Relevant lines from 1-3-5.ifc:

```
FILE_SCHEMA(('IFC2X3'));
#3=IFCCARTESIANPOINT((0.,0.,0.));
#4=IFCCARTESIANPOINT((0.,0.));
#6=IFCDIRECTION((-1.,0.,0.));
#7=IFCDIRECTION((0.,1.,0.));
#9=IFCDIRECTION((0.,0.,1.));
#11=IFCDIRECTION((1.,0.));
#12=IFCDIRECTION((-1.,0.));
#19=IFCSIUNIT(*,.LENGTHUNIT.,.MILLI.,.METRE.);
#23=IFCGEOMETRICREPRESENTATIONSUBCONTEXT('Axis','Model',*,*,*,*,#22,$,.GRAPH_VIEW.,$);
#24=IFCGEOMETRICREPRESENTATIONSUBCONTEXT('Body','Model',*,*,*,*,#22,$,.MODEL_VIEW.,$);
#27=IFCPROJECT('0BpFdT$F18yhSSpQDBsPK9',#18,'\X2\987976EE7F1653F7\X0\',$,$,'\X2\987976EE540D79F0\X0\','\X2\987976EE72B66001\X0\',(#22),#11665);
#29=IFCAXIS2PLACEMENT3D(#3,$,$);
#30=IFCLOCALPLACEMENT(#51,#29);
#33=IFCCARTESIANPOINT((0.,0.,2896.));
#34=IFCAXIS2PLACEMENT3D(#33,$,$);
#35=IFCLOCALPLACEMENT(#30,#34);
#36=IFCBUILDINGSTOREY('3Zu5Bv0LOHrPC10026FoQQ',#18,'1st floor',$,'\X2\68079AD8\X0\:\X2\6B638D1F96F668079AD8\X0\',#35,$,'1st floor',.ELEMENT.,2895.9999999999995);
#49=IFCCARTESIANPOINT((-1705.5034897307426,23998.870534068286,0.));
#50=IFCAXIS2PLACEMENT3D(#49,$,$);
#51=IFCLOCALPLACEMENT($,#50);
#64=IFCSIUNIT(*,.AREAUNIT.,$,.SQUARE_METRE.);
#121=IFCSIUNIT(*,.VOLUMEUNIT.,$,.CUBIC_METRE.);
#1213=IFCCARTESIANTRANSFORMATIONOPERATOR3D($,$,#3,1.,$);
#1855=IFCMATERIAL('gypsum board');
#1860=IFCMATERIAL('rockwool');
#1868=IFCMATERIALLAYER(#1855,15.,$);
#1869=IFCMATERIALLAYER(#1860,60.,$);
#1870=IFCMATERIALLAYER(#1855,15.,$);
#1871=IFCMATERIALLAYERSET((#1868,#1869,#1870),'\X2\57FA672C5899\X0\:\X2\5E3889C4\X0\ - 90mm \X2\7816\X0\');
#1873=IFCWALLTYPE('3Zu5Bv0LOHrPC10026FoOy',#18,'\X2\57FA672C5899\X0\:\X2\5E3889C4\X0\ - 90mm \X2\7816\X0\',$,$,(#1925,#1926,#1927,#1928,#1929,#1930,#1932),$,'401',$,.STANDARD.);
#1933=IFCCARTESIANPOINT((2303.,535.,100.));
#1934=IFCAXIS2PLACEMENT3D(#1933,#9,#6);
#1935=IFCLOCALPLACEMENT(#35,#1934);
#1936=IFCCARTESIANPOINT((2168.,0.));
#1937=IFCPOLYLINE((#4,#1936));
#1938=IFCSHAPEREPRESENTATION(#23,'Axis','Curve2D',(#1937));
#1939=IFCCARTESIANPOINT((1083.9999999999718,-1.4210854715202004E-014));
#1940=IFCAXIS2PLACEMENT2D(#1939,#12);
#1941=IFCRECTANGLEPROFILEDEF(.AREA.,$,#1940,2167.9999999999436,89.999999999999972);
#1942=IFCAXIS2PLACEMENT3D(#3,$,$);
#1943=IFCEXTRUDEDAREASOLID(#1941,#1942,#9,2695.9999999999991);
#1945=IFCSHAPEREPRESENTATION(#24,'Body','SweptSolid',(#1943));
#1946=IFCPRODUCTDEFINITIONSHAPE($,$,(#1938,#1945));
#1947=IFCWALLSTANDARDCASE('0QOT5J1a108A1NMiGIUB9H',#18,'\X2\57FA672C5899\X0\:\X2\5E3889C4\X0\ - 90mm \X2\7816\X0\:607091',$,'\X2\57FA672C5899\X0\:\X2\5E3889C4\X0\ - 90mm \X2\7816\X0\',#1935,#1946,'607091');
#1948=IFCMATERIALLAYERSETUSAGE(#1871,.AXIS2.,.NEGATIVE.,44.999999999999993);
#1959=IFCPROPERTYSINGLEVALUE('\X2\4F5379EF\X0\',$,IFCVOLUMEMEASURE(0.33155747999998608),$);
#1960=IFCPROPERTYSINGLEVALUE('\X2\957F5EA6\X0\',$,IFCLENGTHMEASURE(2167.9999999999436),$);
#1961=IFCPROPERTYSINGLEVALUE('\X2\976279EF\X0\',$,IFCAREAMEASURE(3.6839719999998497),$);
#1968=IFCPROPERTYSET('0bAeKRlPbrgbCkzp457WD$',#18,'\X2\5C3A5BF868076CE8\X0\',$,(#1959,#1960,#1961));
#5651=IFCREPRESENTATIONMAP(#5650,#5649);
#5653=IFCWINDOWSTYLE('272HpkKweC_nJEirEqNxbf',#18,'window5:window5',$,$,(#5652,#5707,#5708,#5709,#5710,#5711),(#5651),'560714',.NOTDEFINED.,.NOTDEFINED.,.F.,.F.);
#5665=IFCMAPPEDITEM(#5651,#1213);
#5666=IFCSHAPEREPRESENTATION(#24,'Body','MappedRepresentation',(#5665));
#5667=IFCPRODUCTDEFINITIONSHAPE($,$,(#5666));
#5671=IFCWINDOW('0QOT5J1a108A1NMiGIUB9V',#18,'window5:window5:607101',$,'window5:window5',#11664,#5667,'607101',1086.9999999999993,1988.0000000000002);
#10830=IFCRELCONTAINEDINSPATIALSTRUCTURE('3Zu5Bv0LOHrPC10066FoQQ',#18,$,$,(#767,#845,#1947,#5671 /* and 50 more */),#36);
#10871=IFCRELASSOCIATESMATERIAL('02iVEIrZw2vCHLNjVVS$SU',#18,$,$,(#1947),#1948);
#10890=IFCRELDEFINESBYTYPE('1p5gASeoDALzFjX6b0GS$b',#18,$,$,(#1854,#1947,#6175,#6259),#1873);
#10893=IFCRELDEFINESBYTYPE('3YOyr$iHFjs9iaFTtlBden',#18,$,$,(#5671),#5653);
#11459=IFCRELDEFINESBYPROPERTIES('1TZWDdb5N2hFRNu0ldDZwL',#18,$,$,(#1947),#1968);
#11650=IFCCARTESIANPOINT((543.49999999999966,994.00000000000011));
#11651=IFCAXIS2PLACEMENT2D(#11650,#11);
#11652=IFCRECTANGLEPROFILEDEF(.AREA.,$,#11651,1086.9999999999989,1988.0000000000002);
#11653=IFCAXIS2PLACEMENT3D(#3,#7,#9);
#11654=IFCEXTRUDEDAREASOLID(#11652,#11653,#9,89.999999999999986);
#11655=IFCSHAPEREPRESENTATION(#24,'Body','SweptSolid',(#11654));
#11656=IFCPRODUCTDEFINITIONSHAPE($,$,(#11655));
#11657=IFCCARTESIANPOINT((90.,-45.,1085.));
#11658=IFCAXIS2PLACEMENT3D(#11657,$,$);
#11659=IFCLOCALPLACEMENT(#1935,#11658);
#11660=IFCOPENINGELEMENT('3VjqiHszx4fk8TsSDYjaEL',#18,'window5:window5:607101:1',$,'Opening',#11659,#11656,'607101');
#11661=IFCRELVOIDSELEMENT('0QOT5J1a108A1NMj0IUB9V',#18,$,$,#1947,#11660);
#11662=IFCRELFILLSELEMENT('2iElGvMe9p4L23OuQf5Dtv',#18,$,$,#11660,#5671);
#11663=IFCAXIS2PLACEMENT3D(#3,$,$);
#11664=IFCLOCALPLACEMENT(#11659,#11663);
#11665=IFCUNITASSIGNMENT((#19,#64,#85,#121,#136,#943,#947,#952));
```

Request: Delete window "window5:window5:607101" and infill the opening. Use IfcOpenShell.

```python
import ifcopenshell
import ifcopenshell.api.feature
import ifcopenshell.api.pset
import ifcopenshell.api.root
import ifcopenshell.geom
import ifcopenshell.util.element
import ifcopenshell.util.shape
import ifcopenshell.util.unit

model = ifcopenshell.open("1-3-5.ifc")
area_scale = ifcopenshell.util.unit.calculate_unit_scale(model, "AREAUNIT")
volume_scale = ifcopenshell.util.unit.calculate_unit_scale(model, "VOLUMEUNIT")
settings = ifcopenshell.geom.settings()


def volume(element):
    """Net volume in cubic metres, openings subtracted."""
    shape = ifcopenshell.geom.create_shape(settings, element)
    return ifcopenshell.util.shape.get_volume(shape.geometry)


window = model.by_guid("0QOT5J1a108A1NMiGIUB9V")
opening = window.FillsVoids[0].RelatingOpeningElement
wall = opening.VoidsElements[0].RelatingBuildingElement
before = volume(wall)

ifcopenshell.api.root.remove_product(model, product=window)
ifcopenshell.api.feature.remove_feature(model, feature=opening)

after = volume(wall)
thickness = 0.09  # wall thickness in metres

# Update the wall's stored quantities.
pset = model.by_id(ifcopenshell.util.element.get_pset(wall, "尺寸标注", should_inherit=False)["id"])
ifcopenshell.api.pset.edit_pset(model, pset=pset, properties={
    "体积": model.create_entity("IfcVolumeMeasure", after / volume_scale),
    "面积": model.create_entity("IfcAreaMeasure", after / thickness / area_scale),
})

print(f"wall volume {before:.3f} -> {after:.3f} m3")

model.write("1-3-5_v2.ifc")
```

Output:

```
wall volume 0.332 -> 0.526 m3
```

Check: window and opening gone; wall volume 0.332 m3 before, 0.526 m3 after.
